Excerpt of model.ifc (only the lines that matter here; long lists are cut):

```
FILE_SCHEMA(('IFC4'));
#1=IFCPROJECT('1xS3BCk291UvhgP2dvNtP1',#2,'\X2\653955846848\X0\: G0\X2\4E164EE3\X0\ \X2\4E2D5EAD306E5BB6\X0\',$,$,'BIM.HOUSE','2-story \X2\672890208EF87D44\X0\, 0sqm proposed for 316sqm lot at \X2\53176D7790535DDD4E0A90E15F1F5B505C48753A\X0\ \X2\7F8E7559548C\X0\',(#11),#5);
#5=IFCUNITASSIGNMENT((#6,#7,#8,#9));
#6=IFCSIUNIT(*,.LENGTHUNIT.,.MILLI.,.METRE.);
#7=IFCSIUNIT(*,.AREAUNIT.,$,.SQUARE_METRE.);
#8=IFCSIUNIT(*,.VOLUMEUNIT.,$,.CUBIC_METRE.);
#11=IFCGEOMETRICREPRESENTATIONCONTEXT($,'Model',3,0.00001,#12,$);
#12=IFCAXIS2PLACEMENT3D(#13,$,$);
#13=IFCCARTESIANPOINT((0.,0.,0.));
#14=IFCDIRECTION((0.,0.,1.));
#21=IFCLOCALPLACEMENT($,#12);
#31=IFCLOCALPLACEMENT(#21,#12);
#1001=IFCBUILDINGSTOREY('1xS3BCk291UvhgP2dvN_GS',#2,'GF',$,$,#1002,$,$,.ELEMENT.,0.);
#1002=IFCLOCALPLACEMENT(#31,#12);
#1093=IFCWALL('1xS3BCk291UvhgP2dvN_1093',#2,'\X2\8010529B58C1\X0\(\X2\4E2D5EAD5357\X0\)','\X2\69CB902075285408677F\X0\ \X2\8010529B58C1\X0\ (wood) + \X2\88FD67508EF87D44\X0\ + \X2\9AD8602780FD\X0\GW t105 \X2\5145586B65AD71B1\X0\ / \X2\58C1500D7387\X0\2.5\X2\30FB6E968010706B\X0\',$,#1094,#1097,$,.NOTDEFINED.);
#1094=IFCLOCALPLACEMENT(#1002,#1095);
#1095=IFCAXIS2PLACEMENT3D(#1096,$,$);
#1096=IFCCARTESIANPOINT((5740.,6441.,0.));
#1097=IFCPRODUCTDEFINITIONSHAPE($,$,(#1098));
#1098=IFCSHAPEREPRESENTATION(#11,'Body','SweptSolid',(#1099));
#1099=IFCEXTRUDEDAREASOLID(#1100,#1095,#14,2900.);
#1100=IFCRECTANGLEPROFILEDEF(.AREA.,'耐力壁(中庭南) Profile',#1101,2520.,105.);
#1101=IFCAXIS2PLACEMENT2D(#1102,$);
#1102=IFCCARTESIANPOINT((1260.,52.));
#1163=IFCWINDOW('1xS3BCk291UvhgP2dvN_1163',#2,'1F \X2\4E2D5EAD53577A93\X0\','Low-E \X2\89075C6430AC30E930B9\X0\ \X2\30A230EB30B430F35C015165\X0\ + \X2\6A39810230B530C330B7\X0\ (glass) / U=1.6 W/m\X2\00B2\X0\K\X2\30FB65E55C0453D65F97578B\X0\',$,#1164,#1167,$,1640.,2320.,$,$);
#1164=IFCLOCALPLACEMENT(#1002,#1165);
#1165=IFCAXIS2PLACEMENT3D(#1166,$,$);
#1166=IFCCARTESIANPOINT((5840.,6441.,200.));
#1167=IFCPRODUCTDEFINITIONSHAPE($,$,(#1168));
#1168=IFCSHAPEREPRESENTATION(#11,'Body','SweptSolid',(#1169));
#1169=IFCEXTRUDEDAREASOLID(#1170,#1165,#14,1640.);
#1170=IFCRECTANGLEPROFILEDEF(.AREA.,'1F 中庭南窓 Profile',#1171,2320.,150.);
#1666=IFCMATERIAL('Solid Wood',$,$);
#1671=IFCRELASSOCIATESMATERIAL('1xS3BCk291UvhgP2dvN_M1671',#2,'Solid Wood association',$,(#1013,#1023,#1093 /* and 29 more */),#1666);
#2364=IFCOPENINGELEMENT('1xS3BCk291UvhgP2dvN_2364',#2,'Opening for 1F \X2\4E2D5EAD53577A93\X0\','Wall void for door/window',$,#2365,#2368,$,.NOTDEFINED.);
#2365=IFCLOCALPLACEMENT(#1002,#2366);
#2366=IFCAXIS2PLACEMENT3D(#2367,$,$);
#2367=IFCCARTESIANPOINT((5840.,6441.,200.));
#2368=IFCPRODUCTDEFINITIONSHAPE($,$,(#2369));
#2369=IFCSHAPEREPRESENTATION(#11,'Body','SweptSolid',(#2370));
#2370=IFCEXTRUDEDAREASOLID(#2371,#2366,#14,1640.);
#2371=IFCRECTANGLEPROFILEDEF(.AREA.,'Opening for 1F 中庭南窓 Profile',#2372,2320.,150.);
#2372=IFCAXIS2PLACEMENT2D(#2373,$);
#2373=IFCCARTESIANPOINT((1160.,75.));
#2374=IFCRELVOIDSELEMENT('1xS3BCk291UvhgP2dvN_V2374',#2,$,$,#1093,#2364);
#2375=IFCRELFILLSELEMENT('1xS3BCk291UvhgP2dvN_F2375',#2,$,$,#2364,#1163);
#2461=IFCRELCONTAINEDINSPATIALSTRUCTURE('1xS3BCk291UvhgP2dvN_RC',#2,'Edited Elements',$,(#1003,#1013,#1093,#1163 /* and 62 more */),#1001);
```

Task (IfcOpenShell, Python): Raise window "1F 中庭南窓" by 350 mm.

```python
import numpy as np
import ifcopenshell
import ifcopenshell.api.geometry
import ifcopenshell.util.placement
import ifcopenshell.util.unit

model = ifcopenshell.open("model.ifc")
unit_scale = ifcopenshell.util.unit.calculate_unit_scale(model)

window = model.by_id(1163)
opening = window.FillsVoids[0].RelatingOpeningElement
dz = 0.35 / unit_scale

shift = np.array([0.0, 0.0, dz])
# The window is not placed relative to its opening, so move both.
for product in (opening, window):
    matrix = ifcopenshell.util.placement.get_local_placement(product.ObjectPlacement)
    matrix[:3, 3] += shift
    ifcopenshell.api.geometry.edit_object_placement(model, product=product, matrix=matrix, is_si=False)

print(f"moved by {dz * unit_scale:+.3f} m")

model.write("model_rev.ifc")
```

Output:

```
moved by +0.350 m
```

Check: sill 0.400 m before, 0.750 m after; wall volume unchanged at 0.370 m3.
